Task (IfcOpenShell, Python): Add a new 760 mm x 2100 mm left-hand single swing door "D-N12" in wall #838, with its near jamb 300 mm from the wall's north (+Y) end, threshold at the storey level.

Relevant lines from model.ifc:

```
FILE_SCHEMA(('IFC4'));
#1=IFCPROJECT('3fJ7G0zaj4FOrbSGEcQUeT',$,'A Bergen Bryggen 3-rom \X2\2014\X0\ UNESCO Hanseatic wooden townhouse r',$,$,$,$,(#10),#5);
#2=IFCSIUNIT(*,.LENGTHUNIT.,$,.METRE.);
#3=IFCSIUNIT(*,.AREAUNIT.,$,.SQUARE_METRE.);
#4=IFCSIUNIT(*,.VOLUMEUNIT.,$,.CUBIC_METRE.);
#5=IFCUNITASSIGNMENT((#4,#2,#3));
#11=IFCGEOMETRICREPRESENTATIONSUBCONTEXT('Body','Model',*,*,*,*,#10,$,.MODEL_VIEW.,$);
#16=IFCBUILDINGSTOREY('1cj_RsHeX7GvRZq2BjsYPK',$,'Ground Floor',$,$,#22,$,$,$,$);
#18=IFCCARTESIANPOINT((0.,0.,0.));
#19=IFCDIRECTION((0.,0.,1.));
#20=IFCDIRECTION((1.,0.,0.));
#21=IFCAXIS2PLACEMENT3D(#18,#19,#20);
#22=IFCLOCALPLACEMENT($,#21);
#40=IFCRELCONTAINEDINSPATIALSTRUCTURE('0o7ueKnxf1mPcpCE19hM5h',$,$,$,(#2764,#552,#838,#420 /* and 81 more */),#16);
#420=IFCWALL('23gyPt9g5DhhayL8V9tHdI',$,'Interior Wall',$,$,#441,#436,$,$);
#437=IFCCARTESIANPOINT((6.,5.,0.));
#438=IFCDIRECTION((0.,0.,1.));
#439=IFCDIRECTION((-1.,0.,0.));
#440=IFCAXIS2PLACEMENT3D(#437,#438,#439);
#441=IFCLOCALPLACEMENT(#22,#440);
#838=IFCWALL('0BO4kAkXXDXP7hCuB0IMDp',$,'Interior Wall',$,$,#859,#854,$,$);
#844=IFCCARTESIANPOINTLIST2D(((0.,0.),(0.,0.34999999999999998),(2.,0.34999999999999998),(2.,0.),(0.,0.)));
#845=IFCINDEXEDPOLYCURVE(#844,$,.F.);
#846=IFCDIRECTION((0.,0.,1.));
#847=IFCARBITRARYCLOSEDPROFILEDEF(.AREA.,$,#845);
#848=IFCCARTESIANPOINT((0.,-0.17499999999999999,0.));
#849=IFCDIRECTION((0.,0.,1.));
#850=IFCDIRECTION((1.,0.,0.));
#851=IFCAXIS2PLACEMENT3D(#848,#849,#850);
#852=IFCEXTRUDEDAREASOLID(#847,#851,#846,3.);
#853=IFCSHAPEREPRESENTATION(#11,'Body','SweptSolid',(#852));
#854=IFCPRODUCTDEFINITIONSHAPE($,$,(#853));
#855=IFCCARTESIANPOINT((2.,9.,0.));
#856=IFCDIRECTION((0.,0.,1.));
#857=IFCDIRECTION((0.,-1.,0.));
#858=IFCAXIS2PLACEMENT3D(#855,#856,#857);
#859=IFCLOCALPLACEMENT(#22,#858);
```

```python
import numpy as np
import ifcopenshell
import ifcopenshell.api.feature
import ifcopenshell.api.geometry
import ifcopenshell.api.root
import ifcopenshell.api.spatial
import ifcopenshell.geom
import ifcopenshell.util.element
import ifcopenshell.util.placement
import ifcopenshell.util.representation
import ifcopenshell.util.shape
import ifcopenshell.util.unit

model = ifcopenshell.open("model.ifc")
unit_scale = ifcopenshell.util.unit.calculate_unit_scale(model)
settings = ifcopenshell.geom.settings()


def volume(element):
    """Net volume in cubic metres, openings subtracted."""
    shape = ifcopenshell.geom.create_shape(settings, element)
    return ifcopenshell.util.shape.get_volume(shape.geometry)


wall = model.by_id(838)
storey = ifcopenshell.util.element.get_container(wall, ifc_class="IfcBuildingStorey")
context = ifcopenshell.util.representation.get_context(model, "Model", "Body", "MODEL_VIEW")
before = volume(wall)

width, height, from_end, sill = 0.76, 2.1, 0.3, 0.0  # metres

# The wall runs along its own X axis, and the end named is its -X end.
wall_shape = ifcopenshell.geom.create_shape(settings, wall)
x, y, z = ifcopenshell.util.shape.get_vertices(wall_shape.geometry).T
start = x.min() + from_end
face, thickness = float(y.min()), float(y.max() - y.min())
wall_matrix = ifcopenshell.util.placement.get_local_placement(wall.ObjectPlacement)
level = ifcopenshell.util.placement.get_local_placement(storey.ObjectPlacement)[2, 3]


def in_wall(x, y):
    """Placement at x, y metres in the wall's axes, at sill height."""
    matrix = wall_matrix.copy()
    matrix[:, 3] = wall_matrix @ np.array([x / unit_scale, y / unit_scale, 0.0, 1.0])
    matrix[2, 3] = level + sill / unit_scale
    return matrix


# Opening: a box that overshoots both wall faces by 50 mm.
opening = ifcopenshell.api.root.create_entity(model, ifc_class="IfcOpeningElement", predefined_type="OPENING")
box = ifcopenshell.api.geometry.add_wall_representation(
    model, context=context, length=width, height=height, thickness=thickness + 0.1
)
ifcopenshell.api.geometry.assign_representation(model, product=opening, representation=box)
ifcopenshell.api.geometry.edit_object_placement(model, product=opening, matrix=in_wall(start, face - 0.05), is_si=False)
ifcopenshell.api.feature.add_feature(model, feature=opening, element=wall)

door = ifcopenshell.api.root.create_entity(model, ifc_class="IfcDoor", name="D-N12", predefined_type="DOOR")
door.OverallWidth, door.OverallHeight = width / unit_scale, height / unit_scale
door.OperationType = "SINGLE_SWING_LEFT"
body = ifcopenshell.api.geometry.add_door_representation(
    model,
    context=context,
    overall_width=door.OverallWidth,
    overall_height=door.OverallHeight,
    operation_type="SINGLE_SWING_LEFT",
    lining_properties={"LiningDepth": thickness / unit_scale, "ThresholdDepth": thickness / unit_scale},
)
ifcopenshell.api.geometry.assign_representation(model, product=door, representation=body)
ifcopenshell.api.spatial.assign_container(model, products=[door], relating_structure=storey)
ifcopenshell.api.feature.add_filling(model, opening=opening, element=door)

# The lining spans the wall, so the door starts at the wall face.
ifcopenshell.api.geometry.edit_object_placement(model, product=door, matrix=in_wall(start, face), is_si=False)

after = volume(wall)

print(f"wall volume {before:.3f} -> {after:.3f} m3")

model.write("model_rev.ifc")
```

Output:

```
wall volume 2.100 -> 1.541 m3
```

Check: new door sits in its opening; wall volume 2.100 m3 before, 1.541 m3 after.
